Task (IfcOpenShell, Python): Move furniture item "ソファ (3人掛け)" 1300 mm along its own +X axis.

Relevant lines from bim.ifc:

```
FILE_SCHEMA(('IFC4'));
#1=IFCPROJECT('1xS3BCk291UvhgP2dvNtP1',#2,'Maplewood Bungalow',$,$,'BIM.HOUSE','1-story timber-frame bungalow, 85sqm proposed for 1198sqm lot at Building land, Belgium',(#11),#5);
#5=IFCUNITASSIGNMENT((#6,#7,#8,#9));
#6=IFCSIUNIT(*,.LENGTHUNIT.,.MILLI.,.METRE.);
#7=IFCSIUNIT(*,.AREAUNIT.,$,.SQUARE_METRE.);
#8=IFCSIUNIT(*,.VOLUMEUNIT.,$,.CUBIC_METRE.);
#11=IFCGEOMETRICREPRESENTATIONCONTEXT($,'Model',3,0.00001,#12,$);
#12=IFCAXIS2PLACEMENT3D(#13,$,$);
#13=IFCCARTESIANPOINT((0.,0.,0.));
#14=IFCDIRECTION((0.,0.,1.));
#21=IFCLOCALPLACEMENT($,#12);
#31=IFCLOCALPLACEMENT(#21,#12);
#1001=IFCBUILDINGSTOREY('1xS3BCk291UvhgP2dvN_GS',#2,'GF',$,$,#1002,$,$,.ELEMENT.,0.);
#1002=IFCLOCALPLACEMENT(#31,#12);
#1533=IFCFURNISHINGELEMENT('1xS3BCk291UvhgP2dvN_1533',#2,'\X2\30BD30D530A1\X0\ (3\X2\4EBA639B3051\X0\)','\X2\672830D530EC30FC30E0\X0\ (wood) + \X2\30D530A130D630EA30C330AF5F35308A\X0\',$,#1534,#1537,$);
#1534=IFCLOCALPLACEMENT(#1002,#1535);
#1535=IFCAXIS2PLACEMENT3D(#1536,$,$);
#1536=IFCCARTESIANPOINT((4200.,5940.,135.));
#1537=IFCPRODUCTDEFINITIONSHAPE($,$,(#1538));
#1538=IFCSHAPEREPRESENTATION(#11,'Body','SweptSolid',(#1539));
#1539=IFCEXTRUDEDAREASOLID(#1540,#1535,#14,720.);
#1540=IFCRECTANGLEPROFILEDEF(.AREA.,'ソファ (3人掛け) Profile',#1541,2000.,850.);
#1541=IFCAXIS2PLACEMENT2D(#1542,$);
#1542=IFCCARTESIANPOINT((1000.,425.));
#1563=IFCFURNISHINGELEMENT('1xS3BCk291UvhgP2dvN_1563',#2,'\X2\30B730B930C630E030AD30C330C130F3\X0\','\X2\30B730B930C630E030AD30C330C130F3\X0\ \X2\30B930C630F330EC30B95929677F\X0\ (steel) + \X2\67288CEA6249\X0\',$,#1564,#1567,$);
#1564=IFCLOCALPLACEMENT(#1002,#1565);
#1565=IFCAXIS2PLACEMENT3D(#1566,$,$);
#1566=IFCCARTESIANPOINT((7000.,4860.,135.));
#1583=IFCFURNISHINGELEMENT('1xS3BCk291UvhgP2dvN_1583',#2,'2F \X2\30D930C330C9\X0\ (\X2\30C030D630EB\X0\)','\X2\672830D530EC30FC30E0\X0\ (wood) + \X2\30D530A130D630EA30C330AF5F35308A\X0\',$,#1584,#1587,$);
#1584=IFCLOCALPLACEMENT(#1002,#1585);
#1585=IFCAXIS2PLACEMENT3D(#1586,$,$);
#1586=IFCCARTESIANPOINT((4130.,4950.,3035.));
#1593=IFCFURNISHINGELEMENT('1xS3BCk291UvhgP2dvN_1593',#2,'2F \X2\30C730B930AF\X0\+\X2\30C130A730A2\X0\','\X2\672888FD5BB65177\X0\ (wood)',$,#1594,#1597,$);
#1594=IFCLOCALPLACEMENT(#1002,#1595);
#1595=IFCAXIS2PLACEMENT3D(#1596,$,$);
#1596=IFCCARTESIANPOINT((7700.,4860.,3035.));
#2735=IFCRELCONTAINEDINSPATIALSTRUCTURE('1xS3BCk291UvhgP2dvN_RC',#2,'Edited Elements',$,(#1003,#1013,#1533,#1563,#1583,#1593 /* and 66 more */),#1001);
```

```python
import ifcopenshell
import ifcopenshell.api.geometry
import ifcopenshell.util.placement

model = ifcopenshell.open("bim.ifc")

item = model.by_guid("1xS3BCk291UvhgP2dvN_1533")
matrix = ifcopenshell.util.placement.get_local_placement(item.ObjectPlacement)
matrix[:3, 3] += matrix[:3, 0] * 1300.0
ifcopenshell.api.geometry.edit_object_placement(model, product=item, matrix=matrix, is_si=False)

print(ifcopenshell.util.placement.get_local_placement(item.ObjectPlacement).round(3) + 0.0)

model.write("bim_edited.ifc")
```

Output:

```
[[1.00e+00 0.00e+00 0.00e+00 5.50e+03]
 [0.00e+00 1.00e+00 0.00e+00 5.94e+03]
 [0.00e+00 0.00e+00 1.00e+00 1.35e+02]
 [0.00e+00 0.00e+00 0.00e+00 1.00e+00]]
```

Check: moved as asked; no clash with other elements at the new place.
